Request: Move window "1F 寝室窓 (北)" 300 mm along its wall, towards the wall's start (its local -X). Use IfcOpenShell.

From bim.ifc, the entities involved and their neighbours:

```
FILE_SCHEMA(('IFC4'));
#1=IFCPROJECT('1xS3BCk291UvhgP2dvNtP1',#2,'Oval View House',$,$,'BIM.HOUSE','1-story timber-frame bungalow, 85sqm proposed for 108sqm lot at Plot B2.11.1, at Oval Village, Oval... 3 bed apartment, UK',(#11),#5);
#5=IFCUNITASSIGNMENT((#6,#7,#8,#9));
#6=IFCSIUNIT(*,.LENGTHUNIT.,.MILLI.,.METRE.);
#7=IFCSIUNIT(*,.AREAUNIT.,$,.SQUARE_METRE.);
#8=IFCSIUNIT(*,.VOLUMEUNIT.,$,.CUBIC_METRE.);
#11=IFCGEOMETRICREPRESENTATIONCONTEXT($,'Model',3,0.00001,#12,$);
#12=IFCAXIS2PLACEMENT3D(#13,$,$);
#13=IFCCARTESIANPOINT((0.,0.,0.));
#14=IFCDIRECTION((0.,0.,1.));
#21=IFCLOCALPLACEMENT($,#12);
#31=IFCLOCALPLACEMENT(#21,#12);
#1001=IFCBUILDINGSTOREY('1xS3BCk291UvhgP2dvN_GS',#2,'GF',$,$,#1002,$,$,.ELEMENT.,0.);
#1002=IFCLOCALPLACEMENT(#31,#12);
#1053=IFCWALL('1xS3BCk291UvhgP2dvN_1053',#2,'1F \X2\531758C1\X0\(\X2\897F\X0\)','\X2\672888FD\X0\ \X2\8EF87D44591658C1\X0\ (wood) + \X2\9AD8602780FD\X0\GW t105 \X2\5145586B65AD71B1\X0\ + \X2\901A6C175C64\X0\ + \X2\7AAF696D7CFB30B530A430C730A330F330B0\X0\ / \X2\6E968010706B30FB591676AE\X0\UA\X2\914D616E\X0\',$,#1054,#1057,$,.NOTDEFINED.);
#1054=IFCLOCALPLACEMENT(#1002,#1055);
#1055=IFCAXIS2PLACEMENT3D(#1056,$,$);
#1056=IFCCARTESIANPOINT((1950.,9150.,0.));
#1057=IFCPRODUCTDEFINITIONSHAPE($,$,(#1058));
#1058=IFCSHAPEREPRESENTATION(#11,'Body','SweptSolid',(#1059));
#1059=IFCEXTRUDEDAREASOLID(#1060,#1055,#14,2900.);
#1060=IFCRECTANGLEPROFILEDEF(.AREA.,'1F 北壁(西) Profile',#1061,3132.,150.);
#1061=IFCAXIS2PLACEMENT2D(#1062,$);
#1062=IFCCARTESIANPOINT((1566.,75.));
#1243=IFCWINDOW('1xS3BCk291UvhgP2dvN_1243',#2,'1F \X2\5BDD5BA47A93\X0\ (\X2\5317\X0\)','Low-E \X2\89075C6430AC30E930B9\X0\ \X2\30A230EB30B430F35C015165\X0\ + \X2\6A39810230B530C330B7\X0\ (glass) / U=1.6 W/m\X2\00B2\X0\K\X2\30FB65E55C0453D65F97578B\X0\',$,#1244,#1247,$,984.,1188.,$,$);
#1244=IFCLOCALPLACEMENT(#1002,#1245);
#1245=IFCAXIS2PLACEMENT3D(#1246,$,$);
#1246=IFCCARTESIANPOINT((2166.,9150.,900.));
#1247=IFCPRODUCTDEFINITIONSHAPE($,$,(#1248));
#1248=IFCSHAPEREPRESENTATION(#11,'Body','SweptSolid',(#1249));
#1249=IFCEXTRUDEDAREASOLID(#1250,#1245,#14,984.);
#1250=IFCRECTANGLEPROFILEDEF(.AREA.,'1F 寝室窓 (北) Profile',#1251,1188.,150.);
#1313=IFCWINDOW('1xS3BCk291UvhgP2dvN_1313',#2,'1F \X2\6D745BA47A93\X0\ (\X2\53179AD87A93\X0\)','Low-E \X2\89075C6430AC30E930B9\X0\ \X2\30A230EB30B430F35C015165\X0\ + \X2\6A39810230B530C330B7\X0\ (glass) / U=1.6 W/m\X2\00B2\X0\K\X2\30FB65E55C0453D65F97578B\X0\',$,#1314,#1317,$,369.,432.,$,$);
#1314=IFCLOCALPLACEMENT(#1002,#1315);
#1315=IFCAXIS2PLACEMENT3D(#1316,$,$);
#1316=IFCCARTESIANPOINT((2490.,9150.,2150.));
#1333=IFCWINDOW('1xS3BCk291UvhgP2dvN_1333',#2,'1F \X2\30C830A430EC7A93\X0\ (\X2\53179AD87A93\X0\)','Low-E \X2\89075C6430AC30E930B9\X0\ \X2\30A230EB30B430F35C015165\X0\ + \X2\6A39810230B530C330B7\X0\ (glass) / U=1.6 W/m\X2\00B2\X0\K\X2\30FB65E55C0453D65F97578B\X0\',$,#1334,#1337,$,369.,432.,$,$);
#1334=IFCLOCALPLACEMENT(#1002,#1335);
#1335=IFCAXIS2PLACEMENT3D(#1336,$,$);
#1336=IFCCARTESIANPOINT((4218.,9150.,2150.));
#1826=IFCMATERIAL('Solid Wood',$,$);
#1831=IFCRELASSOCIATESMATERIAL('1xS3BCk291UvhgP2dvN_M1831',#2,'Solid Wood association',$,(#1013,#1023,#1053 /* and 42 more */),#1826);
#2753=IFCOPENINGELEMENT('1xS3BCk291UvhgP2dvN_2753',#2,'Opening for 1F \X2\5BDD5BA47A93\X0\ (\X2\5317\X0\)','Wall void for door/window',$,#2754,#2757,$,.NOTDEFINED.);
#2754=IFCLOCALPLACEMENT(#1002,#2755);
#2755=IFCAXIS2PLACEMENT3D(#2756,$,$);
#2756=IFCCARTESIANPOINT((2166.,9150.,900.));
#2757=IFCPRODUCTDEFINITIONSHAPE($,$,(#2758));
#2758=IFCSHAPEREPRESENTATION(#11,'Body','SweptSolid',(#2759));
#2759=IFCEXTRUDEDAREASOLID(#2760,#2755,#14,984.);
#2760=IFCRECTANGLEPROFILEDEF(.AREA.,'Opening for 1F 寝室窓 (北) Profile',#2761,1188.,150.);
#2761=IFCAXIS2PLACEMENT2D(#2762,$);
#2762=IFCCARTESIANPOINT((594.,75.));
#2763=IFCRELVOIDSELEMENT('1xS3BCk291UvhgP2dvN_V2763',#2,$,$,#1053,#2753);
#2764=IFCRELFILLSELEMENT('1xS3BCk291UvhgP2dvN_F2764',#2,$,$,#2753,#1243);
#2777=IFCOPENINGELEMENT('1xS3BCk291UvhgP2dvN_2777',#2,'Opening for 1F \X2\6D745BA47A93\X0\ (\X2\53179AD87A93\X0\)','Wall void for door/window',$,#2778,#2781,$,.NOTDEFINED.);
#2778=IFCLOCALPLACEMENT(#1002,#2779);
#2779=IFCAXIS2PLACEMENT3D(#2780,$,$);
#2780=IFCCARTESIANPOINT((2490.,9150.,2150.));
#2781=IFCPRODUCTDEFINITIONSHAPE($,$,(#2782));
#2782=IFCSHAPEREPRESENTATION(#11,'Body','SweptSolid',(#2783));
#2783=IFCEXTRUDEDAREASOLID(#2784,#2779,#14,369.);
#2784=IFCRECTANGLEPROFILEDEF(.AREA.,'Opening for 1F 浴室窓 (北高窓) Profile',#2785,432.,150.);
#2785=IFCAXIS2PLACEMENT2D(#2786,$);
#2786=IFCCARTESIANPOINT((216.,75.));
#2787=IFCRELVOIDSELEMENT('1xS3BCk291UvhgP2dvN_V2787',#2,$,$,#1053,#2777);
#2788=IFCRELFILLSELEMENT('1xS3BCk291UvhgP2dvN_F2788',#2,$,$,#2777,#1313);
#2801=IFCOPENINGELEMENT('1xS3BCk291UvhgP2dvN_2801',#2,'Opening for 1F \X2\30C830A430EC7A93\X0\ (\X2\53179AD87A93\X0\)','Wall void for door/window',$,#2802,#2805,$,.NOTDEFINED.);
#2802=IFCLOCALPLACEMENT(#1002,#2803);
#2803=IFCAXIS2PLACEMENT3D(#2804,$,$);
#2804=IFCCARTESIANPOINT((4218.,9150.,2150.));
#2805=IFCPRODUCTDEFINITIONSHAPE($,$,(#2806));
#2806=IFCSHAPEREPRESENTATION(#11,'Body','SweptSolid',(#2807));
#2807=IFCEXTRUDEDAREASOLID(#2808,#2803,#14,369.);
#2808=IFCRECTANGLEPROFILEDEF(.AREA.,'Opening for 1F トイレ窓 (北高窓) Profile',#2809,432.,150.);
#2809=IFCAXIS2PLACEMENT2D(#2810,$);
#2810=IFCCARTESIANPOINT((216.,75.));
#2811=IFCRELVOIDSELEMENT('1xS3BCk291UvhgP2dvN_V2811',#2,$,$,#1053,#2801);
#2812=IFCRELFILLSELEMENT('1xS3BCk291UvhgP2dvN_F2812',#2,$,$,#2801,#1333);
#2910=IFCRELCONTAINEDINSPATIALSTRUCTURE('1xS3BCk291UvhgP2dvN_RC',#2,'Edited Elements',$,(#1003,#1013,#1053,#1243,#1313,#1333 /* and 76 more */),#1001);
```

```python
import ifcopenshell
import ifcopenshell.api.geometry
import ifcopenshell.util.placement

model = ifcopenshell.open("bim.ifc")

window = model.by_guid("1xS3BCk291UvhgP2dvN_1243")
opening = window.FillsVoids[0].RelatingOpeningElement
wall = opening.VoidsElements[0].RelatingBuildingElement

wall_matrix = ifcopenshell.util.placement.get_local_placement(wall.ObjectPlacement)
shift = wall_matrix[:3, 0] * -300.0
before = ifcopenshell.util.placement.get_local_placement(window.ObjectPlacement)[:3, 3].copy()

# The window is not placed relative to its opening, so move both.
for product in (opening, window):
    matrix = ifcopenshell.util.placement.get_local_placement(product.ObjectPlacement)
    matrix[:3, 3] += shift
    ifcopenshell.api.geometry.edit_object_placement(model, product=product, matrix=matrix, is_si=False)

after = ifcopenshell.util.placement.get_local_placement(window.ObjectPlacement)[:3, 3]
print("window moved by", (after - before).round(3) + 0.0)

model.write("bim-out.ifc")
```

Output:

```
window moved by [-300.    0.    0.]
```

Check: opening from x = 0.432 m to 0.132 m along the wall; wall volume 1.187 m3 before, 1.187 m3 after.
